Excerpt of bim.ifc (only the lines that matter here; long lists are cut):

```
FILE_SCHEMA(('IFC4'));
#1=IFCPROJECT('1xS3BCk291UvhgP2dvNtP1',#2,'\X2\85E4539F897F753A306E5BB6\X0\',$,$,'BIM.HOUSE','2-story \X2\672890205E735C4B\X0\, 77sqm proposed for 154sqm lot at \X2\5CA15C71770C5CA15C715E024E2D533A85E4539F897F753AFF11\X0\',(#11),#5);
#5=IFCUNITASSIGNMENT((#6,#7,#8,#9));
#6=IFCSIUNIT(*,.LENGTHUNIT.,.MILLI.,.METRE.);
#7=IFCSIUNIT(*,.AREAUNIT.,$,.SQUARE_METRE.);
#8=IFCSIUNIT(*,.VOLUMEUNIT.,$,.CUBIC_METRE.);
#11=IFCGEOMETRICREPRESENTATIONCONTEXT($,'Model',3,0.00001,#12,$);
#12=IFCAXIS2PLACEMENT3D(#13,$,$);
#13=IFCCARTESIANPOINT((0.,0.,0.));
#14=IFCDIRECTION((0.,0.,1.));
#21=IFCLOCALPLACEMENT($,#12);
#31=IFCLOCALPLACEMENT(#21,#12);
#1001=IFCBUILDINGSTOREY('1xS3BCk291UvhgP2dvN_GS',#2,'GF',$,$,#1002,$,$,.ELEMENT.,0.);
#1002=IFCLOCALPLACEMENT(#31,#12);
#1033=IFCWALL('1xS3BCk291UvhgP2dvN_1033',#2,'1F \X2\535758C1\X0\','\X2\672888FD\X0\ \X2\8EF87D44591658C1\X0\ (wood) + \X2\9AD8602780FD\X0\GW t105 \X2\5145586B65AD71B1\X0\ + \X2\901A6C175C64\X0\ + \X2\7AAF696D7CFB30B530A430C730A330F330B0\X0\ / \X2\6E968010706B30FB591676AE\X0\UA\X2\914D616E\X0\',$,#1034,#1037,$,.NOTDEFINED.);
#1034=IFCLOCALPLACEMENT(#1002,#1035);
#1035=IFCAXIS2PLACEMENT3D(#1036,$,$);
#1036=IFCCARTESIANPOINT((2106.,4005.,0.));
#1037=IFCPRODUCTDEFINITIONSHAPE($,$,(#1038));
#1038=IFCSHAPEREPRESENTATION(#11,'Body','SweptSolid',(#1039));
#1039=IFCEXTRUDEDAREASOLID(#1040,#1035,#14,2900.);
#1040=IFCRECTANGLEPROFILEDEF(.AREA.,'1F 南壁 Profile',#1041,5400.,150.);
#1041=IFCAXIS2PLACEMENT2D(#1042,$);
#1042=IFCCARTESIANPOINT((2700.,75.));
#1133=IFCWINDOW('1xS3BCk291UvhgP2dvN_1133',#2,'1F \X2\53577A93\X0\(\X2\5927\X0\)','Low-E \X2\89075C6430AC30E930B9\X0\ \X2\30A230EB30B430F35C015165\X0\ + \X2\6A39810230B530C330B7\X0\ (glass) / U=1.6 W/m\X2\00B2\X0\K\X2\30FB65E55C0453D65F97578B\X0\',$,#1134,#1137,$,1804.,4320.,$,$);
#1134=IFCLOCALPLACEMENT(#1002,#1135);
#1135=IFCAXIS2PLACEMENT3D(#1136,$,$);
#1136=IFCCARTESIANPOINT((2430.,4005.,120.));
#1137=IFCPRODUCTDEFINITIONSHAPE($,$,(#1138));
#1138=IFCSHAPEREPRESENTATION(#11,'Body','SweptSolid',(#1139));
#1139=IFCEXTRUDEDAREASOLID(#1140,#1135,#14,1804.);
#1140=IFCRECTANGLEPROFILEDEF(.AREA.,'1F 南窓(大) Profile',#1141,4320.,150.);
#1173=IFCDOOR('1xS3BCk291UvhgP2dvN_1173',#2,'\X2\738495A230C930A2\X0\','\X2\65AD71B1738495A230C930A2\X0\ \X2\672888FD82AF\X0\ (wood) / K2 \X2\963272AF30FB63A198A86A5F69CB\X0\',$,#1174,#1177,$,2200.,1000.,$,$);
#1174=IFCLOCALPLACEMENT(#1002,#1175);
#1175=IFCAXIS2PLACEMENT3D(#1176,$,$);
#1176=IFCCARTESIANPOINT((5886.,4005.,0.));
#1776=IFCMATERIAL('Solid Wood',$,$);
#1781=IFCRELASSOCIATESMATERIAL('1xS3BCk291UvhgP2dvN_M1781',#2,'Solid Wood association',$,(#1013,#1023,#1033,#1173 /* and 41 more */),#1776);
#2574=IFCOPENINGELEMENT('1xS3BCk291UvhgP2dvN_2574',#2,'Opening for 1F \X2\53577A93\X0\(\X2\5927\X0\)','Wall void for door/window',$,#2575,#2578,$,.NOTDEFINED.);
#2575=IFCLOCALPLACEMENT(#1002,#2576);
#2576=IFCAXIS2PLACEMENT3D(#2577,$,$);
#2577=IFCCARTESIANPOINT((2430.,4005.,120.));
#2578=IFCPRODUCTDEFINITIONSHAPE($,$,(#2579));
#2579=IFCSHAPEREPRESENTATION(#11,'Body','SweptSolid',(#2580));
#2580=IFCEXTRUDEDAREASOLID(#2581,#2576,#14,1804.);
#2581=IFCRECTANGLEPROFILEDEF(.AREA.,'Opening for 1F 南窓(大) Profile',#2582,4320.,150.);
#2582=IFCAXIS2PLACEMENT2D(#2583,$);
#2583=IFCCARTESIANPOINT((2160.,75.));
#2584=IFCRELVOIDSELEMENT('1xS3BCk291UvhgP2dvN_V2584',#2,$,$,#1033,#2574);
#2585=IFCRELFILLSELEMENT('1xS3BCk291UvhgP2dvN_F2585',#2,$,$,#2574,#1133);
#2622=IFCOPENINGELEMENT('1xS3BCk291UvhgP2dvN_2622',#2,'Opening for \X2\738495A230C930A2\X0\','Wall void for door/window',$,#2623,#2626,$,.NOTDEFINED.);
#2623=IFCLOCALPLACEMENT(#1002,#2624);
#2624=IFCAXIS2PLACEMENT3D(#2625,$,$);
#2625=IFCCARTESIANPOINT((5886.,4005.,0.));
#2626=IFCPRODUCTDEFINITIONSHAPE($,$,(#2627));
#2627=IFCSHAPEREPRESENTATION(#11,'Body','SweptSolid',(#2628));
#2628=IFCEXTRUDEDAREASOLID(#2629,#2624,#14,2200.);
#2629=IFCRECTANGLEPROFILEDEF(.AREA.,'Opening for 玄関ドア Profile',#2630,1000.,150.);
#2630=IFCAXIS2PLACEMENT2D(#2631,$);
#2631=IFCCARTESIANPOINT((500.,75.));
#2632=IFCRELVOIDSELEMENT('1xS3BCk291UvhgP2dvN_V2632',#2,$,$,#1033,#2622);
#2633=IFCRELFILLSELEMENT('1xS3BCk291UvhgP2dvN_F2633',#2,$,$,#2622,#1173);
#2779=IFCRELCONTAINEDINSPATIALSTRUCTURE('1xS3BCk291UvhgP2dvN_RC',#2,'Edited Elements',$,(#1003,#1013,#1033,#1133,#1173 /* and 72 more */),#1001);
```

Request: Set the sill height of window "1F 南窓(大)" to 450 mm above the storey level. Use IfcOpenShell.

```python
import numpy as np
import ifcopenshell
import ifcopenshell.api.geometry
import ifcopenshell.geom
import ifcopenshell.util.element
import ifcopenshell.util.placement
import ifcopenshell.util.shape
import ifcopenshell.util.unit

model = ifcopenshell.open("bim.ifc")
unit_scale = ifcopenshell.util.unit.calculate_unit_scale(model)

window = model.by_guid("1xS3BCk291UvhgP2dvN_1133")
opening = window.FillsVoids[0].RelatingOpeningElement
storey = ifcopenshell.util.element.get_container(window, ifc_class="IfcBuildingStorey")
level = ifcopenshell.util.placement.get_local_placement(storey.ObjectPlacement)[2, 3]

# The opening's origin need not be at the sill, so measure its lowest point.
shape = ifcopenshell.geom.create_shape(ifcopenshell.geom.settings(), opening)
bottom = ifcopenshell.util.shape.get_shape_bottom_elevation(shape, shape.geometry) / unit_scale
dz = level + 0.45 / unit_scale - bottom

shift = np.array([0.0, 0.0, dz])
# The window is not placed relative to its opening, so move both.
for product in (opening, window):
    matrix = ifcopenshell.util.placement.get_local_placement(product.ObjectPlacement)
    matrix[:3, 3] += shift
    ifcopenshell.api.geometry.edit_object_placement(model, product=product, matrix=matrix, is_si=False)

print(f"moved by {dz * unit_scale:+.3f} m")

model.write("bim_v2.ifc")
```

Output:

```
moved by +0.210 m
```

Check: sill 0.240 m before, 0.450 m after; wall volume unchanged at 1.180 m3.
